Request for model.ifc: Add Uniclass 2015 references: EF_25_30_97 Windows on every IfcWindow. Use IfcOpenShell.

First a look at what the model holds.

```python
import ifcopenshell

model = ifcopenshell.open("model.ifc")
print(model.schema)
print("classifications:", [c.Name for c in model.by_type("IfcClassification")])
for ifc_class in ("IfcDoor", "IfcRoof", "IfcStair", "IfcWall", "IfcWindow"):
    print(ifc_class, len(model.by_type(ifc_class)))
```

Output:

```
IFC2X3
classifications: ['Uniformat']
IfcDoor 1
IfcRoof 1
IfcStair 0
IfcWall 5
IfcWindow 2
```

```python
import ifcopenshell
import ifcopenshell.api.classification

model = ifcopenshell.open("model.ifc")

# IFC2X3 requires Source and Edition and has no link from the project to the system.
system = model.create_entity("IfcClassification", Source="NBS", Edition="2015", Name="Uniclass 2015")

codes = {
    "IfcWindow": ("EF_25_30_97", "Windows"),
}
for ifc_class, (code, name) in codes.items():
    products = model.by_type(ifc_class)
    ifcopenshell.api.classification.add_reference(
        model, products=products, classification=system, identification=code, name=name
    )
    print(code, len(products))

model.write("model_v2.ifc")
```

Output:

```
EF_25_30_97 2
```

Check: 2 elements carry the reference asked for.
